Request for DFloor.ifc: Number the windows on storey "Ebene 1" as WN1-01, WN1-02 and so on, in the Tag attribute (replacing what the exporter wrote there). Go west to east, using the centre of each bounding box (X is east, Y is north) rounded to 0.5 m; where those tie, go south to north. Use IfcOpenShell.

First a look at what the model holds.

```python
import ifcopenshell
import ifcopenshell.util.element
import ifcopenshell.util.placement

model = ifcopenshell.open("DFloor.ifc")
print(model.schema)
storey = next(s for s in model.by_type("IfcBuildingStorey") if s.Name == "Ebene 1")
windows = [e for e in ifcopenshell.util.element.get_decomposition(storey) if e.is_a("IfcWindow")]
for e in sorted(windows, key=lambda e: e.id()):
    origin = ifcopenshell.util.placement.get_local_placement(e.ObjectPlacement)[:3, 3]
    print(e.id(), e.Tag, e.Name, origin.round(2) + 0.0, sep=" | ")
```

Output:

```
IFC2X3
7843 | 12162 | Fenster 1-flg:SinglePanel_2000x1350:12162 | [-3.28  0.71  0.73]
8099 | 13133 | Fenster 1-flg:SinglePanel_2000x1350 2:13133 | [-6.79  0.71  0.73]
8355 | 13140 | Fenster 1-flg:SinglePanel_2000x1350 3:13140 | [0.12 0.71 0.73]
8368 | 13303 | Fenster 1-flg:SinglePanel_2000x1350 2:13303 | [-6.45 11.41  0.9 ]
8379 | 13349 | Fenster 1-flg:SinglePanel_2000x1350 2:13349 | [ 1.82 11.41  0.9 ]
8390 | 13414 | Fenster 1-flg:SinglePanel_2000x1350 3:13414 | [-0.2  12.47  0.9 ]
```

```python
import ifcopenshell
import ifcopenshell.geom
import ifcopenshell.util.element
import ifcopenshell.util.shape

model = ifcopenshell.open("DFloor.ifc")
settings = ifcopenshell.geom.settings()
settings.set("use-world-coords", True)


def centre(element):
    shape = ifcopenshell.geom.create_shape(settings, element)
    return ifcopenshell.util.shape.get_bbox_centroid(shape.geometry)


storey = next(s for s in model.by_type("IfcBuildingStorey") if s.Name == "Ebene 1")
windows = [e for e in ifcopenshell.util.element.get_decomposition(storey) if e.is_a("IfcWindow")]

# Insertion points can sit at a corner or the storey origin, so sort by the geometry (in metres).
centres = {e: centre(e) for e in windows}
windows.sort(key=lambda e: (round(centres[e][0] / 0.5), centres[e][1]))

for i, e in enumerate(windows, start=1):
    number = f"WN1-{i:02d}"
    e.Tag = number
    print(e.id(), number)

model.write("DFloor_edited.ifc")
```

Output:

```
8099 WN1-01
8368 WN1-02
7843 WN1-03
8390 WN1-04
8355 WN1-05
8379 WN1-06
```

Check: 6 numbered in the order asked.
